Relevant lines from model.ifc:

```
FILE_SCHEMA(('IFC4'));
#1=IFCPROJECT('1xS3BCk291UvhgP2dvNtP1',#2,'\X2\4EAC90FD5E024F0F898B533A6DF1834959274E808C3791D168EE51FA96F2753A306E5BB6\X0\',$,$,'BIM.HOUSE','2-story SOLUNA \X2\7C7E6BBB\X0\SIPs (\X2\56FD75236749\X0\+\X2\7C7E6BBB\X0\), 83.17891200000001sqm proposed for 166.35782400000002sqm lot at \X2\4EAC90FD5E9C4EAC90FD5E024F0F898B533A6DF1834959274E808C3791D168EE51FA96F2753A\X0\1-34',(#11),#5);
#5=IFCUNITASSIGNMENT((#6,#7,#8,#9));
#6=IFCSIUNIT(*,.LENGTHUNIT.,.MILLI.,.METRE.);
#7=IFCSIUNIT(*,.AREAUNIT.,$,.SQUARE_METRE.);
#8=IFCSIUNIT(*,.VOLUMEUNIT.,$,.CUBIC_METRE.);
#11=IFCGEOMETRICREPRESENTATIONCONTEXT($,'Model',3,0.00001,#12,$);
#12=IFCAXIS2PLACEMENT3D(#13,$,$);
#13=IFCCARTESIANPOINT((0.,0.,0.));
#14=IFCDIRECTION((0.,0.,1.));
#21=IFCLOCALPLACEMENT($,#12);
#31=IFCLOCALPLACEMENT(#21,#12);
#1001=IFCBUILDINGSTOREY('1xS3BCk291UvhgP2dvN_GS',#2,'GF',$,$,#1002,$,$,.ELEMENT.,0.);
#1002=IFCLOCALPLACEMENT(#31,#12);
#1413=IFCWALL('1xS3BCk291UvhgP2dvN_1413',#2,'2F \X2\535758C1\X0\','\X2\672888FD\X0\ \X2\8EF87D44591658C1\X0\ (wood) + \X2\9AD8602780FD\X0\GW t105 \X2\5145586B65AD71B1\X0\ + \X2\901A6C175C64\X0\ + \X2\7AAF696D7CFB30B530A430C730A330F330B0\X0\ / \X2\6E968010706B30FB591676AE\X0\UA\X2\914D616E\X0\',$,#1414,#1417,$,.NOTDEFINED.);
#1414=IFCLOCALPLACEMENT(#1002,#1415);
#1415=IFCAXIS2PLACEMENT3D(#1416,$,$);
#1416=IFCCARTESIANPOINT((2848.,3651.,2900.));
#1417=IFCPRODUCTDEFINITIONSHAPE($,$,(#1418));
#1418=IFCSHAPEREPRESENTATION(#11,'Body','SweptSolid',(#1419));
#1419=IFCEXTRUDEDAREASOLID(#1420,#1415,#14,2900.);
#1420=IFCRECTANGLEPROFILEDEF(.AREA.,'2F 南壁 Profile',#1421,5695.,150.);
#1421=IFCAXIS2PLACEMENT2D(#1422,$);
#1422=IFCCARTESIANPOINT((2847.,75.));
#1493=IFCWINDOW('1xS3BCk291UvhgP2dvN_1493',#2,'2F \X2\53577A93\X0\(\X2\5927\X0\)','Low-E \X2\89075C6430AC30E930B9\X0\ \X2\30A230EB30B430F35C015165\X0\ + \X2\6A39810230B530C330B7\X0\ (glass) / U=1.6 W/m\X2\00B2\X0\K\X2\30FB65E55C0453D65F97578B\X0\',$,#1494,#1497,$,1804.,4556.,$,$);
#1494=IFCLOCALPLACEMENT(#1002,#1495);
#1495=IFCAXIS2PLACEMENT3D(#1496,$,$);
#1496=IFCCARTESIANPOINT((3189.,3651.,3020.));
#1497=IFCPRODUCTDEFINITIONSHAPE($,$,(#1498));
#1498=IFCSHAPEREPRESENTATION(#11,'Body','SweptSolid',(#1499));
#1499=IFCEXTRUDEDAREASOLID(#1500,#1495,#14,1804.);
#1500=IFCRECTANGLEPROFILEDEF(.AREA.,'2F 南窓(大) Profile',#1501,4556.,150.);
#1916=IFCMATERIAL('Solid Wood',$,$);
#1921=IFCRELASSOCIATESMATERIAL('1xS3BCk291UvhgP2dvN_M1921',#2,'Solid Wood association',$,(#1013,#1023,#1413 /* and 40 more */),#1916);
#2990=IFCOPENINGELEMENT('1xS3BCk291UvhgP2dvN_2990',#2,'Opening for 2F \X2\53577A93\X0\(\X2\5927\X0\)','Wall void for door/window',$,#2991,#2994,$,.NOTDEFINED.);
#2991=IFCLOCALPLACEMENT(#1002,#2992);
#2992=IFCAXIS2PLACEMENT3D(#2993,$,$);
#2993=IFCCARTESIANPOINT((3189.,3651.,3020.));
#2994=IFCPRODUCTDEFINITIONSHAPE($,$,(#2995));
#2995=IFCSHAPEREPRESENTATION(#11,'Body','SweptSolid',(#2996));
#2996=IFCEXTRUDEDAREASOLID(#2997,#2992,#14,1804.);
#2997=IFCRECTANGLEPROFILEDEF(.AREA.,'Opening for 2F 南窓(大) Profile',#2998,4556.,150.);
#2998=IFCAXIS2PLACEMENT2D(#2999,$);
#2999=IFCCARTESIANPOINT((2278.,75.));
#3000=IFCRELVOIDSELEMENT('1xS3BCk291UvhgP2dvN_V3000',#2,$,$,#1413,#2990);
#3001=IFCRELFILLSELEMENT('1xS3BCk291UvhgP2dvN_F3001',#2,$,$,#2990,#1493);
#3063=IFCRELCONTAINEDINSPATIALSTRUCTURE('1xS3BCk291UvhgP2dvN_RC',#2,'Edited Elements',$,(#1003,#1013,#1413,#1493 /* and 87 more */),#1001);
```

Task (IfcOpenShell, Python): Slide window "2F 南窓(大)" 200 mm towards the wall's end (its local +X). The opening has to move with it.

```python
import ifcopenshell
import ifcopenshell.api.geometry
import ifcopenshell.util.placement
import ifcopenshell.util.unit

model = ifcopenshell.open("model.ifc")
unit_scale = ifcopenshell.util.unit.calculate_unit_scale(model)

window = model.by_id(1493)
opening = window.FillsVoids[0].RelatingOpeningElement
wall = opening.VoidsElements[0].RelatingBuildingElement

wall_matrix = ifcopenshell.util.placement.get_local_placement(wall.ObjectPlacement)
shift = wall_matrix[:3, 0] * 0.2 / unit_scale
before = ifcopenshell.util.placement.get_local_placement(window.ObjectPlacement)[:3, 3].copy()

# The window is not placed relative to its opening, so move both.
for product in (opening, window):
    matrix = ifcopenshell.util.placement.get_local_placement(product.ObjectPlacement)
    matrix[:3, 3] += shift
    ifcopenshell.api.geometry.edit_object_placement(model, product=product, matrix=matrix, is_si=False)

after = ifcopenshell.util.placement.get_local_placement(window.ObjectPlacement)[:3, 3]
print("window moved by", (after - before).round(3) + 0.0)

model.write("model_rev.ifc")
```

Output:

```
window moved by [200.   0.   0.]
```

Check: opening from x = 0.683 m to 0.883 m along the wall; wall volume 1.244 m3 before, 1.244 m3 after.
